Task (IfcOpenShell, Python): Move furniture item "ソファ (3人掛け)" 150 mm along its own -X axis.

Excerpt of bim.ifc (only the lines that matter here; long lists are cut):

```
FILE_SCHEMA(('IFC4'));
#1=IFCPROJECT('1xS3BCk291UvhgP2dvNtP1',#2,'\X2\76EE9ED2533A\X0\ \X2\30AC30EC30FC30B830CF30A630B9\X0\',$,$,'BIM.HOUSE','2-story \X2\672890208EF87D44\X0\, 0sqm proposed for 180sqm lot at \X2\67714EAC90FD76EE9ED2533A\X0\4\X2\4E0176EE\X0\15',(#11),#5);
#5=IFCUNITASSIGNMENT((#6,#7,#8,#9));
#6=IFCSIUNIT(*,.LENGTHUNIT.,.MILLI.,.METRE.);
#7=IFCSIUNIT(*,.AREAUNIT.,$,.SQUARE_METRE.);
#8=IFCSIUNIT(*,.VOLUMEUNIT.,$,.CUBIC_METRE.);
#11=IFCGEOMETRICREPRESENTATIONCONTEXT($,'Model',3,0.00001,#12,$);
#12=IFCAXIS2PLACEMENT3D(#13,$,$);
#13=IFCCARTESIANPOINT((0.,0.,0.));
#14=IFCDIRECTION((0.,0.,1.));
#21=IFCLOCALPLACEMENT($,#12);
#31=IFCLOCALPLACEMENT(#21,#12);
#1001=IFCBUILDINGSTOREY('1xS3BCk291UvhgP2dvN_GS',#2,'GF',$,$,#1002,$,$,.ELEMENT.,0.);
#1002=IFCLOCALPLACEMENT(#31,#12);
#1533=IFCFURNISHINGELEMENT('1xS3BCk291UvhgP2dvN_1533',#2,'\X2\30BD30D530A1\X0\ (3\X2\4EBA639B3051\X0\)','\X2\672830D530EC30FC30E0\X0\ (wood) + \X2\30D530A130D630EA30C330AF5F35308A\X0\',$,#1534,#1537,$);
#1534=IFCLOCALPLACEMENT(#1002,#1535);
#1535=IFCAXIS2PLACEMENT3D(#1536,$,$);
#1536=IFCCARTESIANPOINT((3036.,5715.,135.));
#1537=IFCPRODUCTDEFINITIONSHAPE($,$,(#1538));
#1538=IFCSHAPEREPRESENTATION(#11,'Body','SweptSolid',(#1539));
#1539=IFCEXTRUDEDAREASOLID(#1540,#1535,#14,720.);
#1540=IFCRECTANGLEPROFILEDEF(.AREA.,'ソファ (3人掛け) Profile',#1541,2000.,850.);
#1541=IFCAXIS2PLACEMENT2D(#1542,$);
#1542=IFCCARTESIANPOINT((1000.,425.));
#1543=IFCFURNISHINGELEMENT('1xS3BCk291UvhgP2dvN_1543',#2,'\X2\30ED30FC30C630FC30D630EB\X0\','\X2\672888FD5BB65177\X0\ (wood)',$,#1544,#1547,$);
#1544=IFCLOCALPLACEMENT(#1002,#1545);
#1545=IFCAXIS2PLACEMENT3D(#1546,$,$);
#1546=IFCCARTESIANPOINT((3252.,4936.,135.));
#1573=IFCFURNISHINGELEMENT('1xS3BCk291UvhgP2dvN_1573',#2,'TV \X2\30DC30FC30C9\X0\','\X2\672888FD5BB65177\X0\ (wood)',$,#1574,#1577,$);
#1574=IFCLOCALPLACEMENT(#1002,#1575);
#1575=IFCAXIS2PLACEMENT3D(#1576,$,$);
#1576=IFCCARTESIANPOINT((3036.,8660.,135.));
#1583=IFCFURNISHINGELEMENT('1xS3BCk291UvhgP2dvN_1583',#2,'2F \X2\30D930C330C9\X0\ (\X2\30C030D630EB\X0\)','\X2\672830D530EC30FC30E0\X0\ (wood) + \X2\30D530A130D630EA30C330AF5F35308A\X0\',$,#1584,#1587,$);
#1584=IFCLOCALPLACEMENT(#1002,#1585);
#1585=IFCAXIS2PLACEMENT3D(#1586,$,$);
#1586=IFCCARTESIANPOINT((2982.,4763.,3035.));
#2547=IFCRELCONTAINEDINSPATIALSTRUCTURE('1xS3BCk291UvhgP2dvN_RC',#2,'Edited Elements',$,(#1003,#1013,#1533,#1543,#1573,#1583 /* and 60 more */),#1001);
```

```python
import ifcopenshell
import ifcopenshell.api.geometry
import ifcopenshell.util.placement
import ifcopenshell.util.unit

model = ifcopenshell.open("bim.ifc")
unit_scale = ifcopenshell.util.unit.calculate_unit_scale(model)

item = model.by_guid("1xS3BCk291UvhgP2dvN_1533")
matrix = ifcopenshell.util.placement.get_local_placement(item.ObjectPlacement)
matrix[:3, 3] -= matrix[:3, 0] * 0.15 / unit_scale
ifcopenshell.api.geometry.edit_object_placement(model, product=item, matrix=matrix, is_si=False)

print(ifcopenshell.util.placement.get_local_placement(item.ObjectPlacement).round(3) + 0.0)

model.write("bim_rev.ifc")
```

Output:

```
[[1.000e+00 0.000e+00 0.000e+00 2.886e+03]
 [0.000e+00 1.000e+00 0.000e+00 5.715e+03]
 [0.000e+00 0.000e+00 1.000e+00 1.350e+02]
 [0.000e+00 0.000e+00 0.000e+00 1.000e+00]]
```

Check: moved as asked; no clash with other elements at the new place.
